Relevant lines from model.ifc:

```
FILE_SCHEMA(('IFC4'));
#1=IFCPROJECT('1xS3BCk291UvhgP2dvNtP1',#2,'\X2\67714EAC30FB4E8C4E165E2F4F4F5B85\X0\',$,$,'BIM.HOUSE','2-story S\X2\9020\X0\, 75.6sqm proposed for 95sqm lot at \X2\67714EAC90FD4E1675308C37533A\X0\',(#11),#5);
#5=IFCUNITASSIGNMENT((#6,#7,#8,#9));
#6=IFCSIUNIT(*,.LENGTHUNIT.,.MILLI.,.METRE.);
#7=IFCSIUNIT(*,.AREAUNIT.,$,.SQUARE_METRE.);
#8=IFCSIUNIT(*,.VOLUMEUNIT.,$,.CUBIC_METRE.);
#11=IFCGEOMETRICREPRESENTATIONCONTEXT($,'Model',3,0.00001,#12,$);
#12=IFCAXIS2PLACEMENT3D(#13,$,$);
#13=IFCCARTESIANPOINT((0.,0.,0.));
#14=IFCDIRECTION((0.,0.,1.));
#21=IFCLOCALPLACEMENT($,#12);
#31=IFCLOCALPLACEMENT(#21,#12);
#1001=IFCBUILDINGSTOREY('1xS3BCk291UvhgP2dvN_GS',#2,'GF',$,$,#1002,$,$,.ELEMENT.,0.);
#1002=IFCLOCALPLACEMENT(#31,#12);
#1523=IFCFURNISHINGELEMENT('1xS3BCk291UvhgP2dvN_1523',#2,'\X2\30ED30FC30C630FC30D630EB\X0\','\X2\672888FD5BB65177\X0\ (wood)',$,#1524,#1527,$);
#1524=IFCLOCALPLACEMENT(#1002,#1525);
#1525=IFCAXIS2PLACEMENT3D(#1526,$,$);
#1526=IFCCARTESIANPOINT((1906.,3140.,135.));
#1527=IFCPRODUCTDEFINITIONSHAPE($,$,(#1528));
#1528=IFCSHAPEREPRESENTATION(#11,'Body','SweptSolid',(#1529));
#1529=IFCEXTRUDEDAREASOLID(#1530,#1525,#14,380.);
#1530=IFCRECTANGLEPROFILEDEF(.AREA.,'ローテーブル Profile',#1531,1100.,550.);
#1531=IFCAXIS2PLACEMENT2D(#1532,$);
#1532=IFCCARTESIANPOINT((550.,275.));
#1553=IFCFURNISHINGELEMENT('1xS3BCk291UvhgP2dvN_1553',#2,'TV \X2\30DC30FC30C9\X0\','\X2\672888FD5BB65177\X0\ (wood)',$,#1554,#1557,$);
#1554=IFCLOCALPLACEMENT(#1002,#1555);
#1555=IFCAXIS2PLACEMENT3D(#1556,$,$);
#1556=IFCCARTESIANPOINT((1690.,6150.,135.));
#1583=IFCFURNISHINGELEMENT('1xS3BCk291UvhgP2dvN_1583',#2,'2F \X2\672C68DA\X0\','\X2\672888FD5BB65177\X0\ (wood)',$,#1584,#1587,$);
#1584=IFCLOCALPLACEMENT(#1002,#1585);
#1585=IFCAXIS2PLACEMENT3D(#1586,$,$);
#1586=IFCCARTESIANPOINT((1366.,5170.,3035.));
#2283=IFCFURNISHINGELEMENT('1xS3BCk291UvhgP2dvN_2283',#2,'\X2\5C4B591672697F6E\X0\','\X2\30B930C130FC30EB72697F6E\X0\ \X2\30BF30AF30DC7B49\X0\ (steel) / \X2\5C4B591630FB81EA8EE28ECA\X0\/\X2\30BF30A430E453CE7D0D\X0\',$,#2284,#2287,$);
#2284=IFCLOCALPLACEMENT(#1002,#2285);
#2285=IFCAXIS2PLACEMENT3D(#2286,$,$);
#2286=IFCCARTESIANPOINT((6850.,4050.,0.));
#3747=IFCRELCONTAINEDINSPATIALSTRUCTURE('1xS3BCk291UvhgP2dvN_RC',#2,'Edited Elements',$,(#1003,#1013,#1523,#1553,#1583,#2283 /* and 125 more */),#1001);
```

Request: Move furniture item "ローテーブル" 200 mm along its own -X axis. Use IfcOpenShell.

```python
import ifcopenshell
import ifcopenshell.api.geometry
import ifcopenshell.util.placement
import ifcopenshell.util.unit

model = ifcopenshell.open("model.ifc")
unit_scale = ifcopenshell.util.unit.calculate_unit_scale(model)

item = model.by_guid("1xS3BCk291UvhgP2dvN_1523")
matrix = ifcopenshell.util.placement.get_local_placement(item.ObjectPlacement)
matrix[:3, 3] -= matrix[:3, 0] * 0.2 / unit_scale
ifcopenshell.api.geometry.edit_object_placement(model, product=item, matrix=matrix, is_si=False)

print(ifcopenshell.util.placement.get_local_placement(item.ObjectPlacement).round(3) + 0.0)

model.write("model-out.ifc")
```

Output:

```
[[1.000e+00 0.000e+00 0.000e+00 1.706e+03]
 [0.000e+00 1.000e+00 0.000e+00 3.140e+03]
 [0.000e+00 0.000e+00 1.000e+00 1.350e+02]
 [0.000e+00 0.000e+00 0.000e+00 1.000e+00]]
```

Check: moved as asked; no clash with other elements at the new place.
